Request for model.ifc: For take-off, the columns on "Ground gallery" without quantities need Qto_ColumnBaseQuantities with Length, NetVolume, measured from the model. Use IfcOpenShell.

First a look at what the model holds.

```python
import ifcopenshell
import ifcopenshell.util.element
import ifcopenshell.util.unit

model = ifcopenshell.open("model.ifc")
print(model.schema)
for unit_type in ("LENGTHUNIT", "AREAUNIT", "VOLUMEUNIT"):
    print(unit_type, ifcopenshell.util.unit.calculate_unit_scale(model, unit_type))
storey = next(s for s in model.by_type("IfcBuildingStorey") if s.Name == "Ground gallery")
columns = [e for e in ifcopenshell.util.element.get_decomposition(storey) if e.is_a("IfcColumn")]
for e in sorted(columns, key=lambda e: e.id()):
    print(e.id(), e.is_a(), e.Name, list(ifcopenshell.util.element.get_psets(e, qtos_only=True)), sep=" | ")
```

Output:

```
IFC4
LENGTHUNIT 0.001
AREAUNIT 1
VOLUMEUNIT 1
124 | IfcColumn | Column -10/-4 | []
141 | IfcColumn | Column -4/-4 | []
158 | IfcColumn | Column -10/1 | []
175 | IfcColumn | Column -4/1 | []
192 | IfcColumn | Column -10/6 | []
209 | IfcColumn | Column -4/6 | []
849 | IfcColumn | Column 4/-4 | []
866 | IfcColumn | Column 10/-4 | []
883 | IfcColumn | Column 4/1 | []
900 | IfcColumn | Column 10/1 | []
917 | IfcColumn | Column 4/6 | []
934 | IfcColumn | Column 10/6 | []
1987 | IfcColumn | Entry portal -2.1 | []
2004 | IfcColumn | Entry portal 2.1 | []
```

```python
import ifcopenshell
import ifcopenshell.api.pset
import ifcopenshell.geom
import ifcopenshell.util.element
import ifcopenshell.util.shape
import ifcopenshell.util.unit

model = ifcopenshell.open("model.ifc")
unit_scale = ifcopenshell.util.unit.calculate_unit_scale(model)
volume_scale = ifcopenshell.util.unit.calculate_unit_scale(model, "VOLUMEUNIT")
settings = ifcopenshell.geom.settings()

storey = next(s for s in model.by_type("IfcBuildingStorey") if s.Name == "Ground gallery")
columns = [e for e in ifcopenshell.util.element.get_decomposition(storey) if e.is_a("IfcColumn")]

for e in sorted(columns, key=lambda e: e.id()):
    if ifcopenshell.util.element.get_psets(e, qtos_only=True, should_inherit=False):
        continue
    # Geometry comes back in metres, in the element's own axes.
    shape = ifcopenshell.geom.create_shape(settings, e)
    values = {
        "Length": ifcopenshell.util.shape.get_z(shape.geometry) / unit_scale,
        "NetVolume": ifcopenshell.util.shape.get_volume(shape.geometry) / volume_scale,
    }
    qto = ifcopenshell.api.pset.add_qto(model, product=e, name="Qto_ColumnBaseQuantities")
    ifcopenshell.api.pset.edit_qto(model, qto=qto, properties=values)
    print(e.id(), {k: round(v, 3) for k, v in values.items()})

model.write("model-out.ifc")
```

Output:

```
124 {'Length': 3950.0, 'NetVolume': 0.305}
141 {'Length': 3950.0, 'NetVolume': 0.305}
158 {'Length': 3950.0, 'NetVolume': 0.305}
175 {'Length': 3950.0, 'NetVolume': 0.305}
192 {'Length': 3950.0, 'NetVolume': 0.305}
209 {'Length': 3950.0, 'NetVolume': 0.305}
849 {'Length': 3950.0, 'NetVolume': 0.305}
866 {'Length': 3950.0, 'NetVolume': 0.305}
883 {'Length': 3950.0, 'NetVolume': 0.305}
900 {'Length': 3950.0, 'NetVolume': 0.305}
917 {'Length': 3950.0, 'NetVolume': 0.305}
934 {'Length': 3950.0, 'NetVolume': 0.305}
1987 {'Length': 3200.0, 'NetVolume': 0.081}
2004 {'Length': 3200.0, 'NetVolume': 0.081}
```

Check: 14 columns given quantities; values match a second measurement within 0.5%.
